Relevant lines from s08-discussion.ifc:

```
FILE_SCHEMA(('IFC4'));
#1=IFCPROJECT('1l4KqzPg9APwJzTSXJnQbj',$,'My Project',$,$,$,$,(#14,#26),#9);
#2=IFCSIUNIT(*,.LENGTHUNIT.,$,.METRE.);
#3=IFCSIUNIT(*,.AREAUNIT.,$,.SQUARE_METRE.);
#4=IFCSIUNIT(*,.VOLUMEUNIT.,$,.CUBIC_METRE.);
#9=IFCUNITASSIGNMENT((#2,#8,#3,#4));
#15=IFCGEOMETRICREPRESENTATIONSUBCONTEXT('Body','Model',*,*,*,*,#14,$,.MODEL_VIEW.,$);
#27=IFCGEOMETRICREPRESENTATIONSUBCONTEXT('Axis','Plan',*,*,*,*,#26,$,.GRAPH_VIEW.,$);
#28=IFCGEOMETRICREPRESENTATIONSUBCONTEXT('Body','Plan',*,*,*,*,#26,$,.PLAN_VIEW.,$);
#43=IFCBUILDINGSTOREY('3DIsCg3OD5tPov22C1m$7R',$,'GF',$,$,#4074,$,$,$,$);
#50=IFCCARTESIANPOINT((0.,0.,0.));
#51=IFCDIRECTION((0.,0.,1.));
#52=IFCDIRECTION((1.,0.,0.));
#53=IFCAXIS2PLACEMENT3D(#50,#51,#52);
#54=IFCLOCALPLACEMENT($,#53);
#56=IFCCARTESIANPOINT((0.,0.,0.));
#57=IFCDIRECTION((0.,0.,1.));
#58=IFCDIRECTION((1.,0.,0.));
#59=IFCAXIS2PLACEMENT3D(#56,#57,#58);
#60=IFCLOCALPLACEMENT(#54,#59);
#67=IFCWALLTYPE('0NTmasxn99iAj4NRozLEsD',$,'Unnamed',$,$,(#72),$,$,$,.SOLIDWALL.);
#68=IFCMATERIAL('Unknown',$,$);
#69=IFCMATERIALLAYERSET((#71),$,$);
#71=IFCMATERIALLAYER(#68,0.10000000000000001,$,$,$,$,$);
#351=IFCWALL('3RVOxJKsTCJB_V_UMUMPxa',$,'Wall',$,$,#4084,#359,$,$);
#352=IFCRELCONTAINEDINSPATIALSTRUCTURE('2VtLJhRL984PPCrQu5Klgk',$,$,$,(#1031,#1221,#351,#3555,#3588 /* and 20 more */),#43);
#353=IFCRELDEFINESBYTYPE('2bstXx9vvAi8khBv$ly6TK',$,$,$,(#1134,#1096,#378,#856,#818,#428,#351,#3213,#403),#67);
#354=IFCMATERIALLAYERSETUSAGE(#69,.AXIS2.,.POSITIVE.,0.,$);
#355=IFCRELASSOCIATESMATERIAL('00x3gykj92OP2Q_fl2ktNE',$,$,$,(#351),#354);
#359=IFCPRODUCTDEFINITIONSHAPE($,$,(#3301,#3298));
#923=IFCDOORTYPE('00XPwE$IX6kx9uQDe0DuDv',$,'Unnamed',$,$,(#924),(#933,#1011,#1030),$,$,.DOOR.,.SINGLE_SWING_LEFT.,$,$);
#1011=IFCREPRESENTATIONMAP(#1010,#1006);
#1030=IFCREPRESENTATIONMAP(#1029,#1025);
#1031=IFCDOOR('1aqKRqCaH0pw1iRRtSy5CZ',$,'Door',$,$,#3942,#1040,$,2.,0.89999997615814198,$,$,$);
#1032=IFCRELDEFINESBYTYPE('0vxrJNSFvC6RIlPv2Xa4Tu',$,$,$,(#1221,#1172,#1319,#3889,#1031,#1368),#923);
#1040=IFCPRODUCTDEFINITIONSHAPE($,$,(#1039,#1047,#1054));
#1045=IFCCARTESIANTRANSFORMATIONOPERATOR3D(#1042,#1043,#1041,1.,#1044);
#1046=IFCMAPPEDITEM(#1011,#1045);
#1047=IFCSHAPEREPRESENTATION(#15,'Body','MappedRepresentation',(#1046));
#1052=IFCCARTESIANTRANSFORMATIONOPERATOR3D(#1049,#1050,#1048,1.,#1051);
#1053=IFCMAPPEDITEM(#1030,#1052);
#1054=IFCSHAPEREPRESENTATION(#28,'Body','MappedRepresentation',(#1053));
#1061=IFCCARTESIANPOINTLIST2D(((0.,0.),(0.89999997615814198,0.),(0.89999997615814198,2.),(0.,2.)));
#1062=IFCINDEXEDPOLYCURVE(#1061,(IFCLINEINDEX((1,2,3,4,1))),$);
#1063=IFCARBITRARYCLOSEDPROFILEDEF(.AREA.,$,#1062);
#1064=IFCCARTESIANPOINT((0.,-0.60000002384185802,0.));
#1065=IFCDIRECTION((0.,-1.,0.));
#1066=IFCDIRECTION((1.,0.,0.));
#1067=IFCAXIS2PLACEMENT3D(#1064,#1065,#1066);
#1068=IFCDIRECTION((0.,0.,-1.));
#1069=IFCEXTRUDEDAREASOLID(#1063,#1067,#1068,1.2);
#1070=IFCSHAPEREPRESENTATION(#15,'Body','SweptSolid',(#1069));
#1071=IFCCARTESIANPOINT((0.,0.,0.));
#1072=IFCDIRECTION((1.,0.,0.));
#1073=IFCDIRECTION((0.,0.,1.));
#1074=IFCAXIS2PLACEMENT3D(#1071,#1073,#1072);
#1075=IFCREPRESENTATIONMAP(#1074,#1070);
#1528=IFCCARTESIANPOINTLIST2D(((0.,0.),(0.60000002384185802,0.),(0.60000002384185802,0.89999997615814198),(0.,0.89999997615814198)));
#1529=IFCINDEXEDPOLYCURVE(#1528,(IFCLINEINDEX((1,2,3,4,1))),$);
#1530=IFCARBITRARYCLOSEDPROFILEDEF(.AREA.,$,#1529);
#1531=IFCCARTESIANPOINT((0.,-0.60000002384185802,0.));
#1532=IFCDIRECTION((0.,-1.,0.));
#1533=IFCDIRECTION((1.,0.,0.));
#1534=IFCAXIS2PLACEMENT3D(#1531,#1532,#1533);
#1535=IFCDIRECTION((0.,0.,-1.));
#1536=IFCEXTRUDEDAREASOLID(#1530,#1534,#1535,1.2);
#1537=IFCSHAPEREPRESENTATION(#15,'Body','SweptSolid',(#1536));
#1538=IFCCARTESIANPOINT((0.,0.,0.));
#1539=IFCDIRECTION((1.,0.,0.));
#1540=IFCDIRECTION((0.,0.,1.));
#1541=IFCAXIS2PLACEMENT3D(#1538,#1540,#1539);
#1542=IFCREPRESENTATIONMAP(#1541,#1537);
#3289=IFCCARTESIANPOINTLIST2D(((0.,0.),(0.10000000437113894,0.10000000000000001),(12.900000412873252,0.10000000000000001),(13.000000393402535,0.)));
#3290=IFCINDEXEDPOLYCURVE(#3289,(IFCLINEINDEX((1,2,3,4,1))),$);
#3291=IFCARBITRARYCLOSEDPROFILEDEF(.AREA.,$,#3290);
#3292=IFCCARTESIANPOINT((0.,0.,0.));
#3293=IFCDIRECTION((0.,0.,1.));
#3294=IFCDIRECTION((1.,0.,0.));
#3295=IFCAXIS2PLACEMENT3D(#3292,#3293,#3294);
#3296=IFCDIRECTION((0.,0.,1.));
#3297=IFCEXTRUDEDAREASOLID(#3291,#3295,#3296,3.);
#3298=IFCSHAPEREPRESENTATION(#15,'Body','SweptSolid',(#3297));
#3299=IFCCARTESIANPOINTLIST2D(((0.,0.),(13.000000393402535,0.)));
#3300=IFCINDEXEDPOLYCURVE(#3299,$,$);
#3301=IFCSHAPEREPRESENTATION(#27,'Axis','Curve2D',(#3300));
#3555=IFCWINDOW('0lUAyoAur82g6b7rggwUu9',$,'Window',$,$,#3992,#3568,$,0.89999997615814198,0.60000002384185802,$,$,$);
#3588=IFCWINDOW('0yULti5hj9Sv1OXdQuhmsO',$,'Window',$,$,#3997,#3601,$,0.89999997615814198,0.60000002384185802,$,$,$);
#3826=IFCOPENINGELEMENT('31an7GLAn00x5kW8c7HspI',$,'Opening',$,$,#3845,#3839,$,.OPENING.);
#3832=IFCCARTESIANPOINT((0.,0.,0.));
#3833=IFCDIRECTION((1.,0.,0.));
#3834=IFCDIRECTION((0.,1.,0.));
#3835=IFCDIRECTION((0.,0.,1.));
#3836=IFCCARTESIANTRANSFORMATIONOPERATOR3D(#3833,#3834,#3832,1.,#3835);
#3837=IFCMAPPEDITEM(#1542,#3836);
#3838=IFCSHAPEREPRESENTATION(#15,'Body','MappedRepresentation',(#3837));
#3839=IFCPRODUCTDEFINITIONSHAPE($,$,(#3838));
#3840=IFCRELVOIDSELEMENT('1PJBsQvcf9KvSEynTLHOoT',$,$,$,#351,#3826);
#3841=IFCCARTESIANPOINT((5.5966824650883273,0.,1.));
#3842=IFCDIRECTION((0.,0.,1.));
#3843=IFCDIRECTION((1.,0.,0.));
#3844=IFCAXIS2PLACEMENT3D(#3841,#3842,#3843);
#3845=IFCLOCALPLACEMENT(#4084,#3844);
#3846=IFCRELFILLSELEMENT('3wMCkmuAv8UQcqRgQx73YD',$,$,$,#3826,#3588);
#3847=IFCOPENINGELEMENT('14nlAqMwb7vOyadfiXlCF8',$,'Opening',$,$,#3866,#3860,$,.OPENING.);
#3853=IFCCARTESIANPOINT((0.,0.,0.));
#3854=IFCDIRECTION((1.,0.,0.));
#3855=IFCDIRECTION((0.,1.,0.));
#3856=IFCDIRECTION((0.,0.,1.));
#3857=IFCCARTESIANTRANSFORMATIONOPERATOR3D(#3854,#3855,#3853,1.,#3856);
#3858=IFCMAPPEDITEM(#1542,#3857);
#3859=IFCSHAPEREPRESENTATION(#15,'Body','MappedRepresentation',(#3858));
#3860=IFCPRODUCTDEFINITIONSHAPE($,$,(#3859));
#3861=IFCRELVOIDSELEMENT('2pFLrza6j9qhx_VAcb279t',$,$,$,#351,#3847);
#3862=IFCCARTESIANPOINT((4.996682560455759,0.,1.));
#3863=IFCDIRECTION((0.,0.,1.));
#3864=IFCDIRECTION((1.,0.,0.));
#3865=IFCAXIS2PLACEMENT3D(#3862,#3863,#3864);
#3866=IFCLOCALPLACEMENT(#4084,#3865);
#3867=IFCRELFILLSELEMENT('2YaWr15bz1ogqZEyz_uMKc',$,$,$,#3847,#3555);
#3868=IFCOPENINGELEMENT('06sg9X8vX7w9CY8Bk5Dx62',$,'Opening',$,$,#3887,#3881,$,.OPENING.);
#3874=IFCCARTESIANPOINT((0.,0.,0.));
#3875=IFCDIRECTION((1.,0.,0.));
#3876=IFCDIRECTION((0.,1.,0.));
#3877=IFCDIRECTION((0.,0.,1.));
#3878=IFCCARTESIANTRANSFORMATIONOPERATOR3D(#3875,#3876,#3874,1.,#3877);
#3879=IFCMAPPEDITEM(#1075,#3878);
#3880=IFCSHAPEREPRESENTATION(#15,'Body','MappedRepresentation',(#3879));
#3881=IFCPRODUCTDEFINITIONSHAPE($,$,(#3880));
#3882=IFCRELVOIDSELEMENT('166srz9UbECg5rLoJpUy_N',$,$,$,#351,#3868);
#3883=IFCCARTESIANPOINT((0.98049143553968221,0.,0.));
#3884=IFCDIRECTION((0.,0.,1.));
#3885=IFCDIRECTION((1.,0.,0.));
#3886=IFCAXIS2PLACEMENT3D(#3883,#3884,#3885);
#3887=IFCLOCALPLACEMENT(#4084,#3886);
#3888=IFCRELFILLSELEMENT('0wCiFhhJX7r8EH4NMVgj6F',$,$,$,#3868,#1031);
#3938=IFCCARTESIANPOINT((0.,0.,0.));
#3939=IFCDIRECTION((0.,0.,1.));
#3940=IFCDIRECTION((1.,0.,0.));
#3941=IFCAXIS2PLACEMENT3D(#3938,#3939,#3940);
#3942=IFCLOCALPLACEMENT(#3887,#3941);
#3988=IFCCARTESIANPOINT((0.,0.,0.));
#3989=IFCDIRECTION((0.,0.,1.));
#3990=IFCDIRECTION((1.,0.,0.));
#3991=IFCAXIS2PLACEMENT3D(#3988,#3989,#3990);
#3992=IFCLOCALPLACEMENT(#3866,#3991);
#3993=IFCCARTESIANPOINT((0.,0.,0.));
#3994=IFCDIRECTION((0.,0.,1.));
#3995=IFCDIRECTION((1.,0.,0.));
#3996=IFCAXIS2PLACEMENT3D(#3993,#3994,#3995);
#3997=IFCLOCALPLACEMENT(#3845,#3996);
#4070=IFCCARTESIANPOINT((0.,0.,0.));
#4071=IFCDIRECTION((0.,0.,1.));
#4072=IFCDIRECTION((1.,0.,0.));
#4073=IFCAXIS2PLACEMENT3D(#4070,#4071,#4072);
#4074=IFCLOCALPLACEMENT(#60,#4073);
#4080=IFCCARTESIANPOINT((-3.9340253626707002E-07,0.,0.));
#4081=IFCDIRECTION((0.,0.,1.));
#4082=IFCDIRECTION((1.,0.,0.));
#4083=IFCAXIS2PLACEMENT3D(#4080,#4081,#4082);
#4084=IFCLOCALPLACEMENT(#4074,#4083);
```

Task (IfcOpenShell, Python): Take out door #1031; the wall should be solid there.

```python
import ifcopenshell
import ifcopenshell.api.feature
import ifcopenshell.api.root
import ifcopenshell.geom
import ifcopenshell.util.shape

model = ifcopenshell.open("s08-discussion.ifc")
settings = ifcopenshell.geom.settings()


def volume(element):
    """Net volume in cubic metres, openings subtracted."""
    shape = ifcopenshell.geom.create_shape(settings, element)
    return ifcopenshell.util.shape.get_volume(shape.geometry)


door = model.by_id(1031)
opening = door.FillsVoids[0].RelatingOpeningElement
wall = opening.VoidsElements[0].RelatingBuildingElement
before = volume(wall)

ifcopenshell.api.root.remove_product(model, product=door)
ifcopenshell.api.feature.remove_feature(model, feature=opening)

after = volume(wall)

print(f"wall volume {before:.3f} -> {after:.3f} m3")

model.write("s08-discussion_edited.ifc")
```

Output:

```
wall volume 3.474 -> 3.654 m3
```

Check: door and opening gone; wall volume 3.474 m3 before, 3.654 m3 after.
